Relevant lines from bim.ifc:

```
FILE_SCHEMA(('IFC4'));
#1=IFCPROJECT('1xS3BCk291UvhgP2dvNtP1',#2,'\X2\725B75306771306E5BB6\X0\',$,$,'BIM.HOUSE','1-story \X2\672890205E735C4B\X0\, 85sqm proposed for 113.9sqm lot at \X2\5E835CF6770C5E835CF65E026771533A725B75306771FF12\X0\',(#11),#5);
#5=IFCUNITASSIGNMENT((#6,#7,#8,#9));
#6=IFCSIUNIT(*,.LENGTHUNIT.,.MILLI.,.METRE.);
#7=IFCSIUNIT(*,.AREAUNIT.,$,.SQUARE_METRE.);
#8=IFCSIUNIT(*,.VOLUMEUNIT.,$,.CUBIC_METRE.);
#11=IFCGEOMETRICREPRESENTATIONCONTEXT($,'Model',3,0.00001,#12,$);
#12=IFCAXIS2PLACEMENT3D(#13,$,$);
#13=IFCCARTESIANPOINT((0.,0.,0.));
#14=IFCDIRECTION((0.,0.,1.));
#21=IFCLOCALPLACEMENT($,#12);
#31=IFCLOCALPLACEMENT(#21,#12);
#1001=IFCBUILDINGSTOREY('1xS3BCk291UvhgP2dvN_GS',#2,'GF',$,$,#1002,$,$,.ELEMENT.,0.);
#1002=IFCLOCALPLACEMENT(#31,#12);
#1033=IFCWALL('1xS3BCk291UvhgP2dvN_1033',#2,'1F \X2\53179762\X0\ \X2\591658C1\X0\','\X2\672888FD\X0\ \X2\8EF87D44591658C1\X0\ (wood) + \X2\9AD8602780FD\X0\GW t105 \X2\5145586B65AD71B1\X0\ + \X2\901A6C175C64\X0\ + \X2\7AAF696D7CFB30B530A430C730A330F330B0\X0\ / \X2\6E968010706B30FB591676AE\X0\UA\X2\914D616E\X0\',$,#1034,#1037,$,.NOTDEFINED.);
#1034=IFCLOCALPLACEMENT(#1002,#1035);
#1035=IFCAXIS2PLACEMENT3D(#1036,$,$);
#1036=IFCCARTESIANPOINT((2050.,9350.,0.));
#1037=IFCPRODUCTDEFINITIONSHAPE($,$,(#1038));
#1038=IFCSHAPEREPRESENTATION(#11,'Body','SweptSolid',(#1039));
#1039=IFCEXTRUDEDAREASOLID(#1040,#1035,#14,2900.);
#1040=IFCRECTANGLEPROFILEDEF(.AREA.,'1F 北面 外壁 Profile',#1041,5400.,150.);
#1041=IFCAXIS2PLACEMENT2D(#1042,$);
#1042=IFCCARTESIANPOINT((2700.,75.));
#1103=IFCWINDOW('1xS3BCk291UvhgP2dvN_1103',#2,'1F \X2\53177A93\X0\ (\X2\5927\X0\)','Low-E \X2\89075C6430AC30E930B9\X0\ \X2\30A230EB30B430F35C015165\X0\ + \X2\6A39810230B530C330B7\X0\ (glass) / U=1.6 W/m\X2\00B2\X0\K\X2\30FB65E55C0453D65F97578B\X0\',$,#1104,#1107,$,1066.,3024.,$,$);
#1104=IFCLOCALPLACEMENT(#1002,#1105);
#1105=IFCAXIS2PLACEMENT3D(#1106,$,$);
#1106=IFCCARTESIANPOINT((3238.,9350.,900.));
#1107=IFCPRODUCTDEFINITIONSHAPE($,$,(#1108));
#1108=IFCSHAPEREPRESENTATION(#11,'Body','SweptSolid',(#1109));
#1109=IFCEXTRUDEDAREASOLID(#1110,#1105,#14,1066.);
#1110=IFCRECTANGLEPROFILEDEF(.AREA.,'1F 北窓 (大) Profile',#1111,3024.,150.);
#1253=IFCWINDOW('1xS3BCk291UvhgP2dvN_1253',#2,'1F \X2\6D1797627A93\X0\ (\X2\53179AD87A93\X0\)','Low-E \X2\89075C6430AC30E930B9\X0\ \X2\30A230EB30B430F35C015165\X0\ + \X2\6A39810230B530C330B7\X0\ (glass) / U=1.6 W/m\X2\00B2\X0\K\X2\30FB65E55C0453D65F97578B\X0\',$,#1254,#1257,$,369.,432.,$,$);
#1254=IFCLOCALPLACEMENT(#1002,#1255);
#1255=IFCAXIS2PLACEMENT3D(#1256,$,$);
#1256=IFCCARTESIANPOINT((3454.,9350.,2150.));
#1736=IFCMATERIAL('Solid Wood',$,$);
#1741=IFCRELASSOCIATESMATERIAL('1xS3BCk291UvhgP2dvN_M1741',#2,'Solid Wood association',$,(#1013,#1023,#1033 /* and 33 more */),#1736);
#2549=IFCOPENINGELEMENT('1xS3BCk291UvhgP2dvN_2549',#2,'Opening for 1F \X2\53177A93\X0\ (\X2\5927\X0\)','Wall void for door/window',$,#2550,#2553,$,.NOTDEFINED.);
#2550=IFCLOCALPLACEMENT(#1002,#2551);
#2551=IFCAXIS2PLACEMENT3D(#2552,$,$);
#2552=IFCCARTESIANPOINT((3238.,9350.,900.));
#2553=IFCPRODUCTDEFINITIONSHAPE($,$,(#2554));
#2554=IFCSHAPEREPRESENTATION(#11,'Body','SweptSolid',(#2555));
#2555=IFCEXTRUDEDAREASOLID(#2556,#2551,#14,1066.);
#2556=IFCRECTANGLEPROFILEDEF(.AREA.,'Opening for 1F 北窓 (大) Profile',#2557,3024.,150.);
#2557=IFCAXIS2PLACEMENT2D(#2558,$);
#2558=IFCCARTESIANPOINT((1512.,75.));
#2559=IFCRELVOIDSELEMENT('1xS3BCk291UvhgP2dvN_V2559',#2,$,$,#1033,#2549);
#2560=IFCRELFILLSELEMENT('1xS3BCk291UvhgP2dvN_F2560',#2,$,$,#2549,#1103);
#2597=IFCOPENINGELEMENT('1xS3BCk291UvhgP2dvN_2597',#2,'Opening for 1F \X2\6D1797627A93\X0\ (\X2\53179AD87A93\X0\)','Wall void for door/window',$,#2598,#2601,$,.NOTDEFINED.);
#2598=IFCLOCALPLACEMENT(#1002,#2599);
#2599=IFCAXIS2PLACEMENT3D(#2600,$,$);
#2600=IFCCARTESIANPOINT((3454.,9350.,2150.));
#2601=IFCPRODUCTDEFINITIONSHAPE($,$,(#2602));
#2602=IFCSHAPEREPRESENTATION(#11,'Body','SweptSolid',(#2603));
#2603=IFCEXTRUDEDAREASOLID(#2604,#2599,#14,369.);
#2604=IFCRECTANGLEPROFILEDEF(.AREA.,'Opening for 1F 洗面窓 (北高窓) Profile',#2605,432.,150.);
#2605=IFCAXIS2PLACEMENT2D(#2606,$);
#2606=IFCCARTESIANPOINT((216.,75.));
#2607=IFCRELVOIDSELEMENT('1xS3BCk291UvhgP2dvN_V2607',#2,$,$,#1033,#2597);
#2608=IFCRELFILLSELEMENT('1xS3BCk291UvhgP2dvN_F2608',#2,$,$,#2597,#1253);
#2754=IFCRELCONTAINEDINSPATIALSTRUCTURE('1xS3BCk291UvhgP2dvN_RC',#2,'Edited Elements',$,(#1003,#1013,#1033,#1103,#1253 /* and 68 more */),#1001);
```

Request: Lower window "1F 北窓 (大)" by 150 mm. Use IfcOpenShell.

```python
import numpy as np
import ifcopenshell
import ifcopenshell.api.geometry
import ifcopenshell.util.placement
import ifcopenshell.util.unit

model = ifcopenshell.open("bim.ifc")
unit_scale = ifcopenshell.util.unit.calculate_unit_scale(model)

window = model.by_guid("1xS3BCk291UvhgP2dvN_1103")
opening = window.FillsVoids[0].RelatingOpeningElement
dz = -0.15 / unit_scale

shift = np.array([0.0, 0.0, dz])
# The window is not placed relative to its opening, so move both.
for product in (opening, window):
    matrix = ifcopenshell.util.placement.get_local_placement(product.ObjectPlacement)
    matrix[:3, 3] += shift
    ifcopenshell.api.geometry.edit_object_placement(model, product=product, matrix=matrix, is_si=False)

print(f"moved by {dz * unit_scale:+.3f} m")

model.write("bim_updated.ifc")
```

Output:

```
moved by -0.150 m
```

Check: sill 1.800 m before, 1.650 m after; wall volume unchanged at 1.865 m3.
